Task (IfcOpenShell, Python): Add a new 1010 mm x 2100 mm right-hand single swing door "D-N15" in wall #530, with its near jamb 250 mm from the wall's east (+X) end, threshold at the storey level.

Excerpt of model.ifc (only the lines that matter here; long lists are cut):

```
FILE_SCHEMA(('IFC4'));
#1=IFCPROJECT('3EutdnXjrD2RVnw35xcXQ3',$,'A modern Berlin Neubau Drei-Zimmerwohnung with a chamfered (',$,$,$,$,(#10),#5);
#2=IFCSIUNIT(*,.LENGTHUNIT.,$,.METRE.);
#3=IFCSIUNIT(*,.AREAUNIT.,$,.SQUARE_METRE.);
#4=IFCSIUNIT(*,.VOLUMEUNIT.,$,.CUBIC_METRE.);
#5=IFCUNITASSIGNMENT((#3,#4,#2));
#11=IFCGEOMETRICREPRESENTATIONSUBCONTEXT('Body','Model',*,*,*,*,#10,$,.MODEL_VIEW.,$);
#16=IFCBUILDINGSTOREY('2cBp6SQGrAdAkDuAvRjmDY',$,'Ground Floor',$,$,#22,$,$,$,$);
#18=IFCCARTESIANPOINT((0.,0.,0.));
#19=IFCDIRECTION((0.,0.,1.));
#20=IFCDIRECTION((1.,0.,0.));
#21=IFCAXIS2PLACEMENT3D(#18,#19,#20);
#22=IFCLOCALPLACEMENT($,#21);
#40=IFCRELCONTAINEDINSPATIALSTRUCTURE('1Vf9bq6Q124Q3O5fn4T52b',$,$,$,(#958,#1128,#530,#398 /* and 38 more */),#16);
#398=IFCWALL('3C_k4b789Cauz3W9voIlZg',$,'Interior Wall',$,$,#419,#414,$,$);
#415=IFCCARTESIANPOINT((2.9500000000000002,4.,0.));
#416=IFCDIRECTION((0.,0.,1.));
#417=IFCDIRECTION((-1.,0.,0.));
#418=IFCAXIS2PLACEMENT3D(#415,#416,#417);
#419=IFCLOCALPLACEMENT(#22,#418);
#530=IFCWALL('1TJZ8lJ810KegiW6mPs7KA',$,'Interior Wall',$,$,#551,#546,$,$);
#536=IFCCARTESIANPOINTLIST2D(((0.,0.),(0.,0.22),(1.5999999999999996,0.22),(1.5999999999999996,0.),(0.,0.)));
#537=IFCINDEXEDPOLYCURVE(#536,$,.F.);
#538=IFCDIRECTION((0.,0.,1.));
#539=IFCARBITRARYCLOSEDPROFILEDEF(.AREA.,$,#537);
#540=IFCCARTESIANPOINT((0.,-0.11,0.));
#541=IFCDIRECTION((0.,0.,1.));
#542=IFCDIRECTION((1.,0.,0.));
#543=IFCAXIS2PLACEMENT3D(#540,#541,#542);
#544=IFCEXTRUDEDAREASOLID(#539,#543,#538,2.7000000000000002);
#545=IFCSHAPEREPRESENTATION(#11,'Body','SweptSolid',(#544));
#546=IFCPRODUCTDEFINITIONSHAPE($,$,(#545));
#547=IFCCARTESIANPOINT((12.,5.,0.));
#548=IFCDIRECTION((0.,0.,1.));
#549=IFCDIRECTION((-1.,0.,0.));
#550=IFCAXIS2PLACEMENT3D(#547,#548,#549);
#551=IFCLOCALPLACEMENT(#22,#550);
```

```python
import numpy as np
import ifcopenshell
import ifcopenshell.api.feature
import ifcopenshell.api.geometry
import ifcopenshell.api.root
import ifcopenshell.api.spatial
import ifcopenshell.geom
import ifcopenshell.util.element
import ifcopenshell.util.placement
import ifcopenshell.util.representation
import ifcopenshell.util.shape
import ifcopenshell.util.unit

model = ifcopenshell.open("model.ifc")
unit_scale = ifcopenshell.util.unit.calculate_unit_scale(model)
settings = ifcopenshell.geom.settings()


def volume(element):
    """Net volume in cubic metres, openings subtracted."""
    shape = ifcopenshell.geom.create_shape(settings, element)
    return ifcopenshell.util.shape.get_volume(shape.geometry)


wall = model.by_id(530)
storey = ifcopenshell.util.element.get_container(wall, ifc_class="IfcBuildingStorey")
context = ifcopenshell.util.representation.get_context(model, "Model", "Body", "MODEL_VIEW")
before = volume(wall)

width, height, from_end, sill = 1.01, 2.1, 0.25, 0.0  # metres

# The wall runs along its own X axis, and the end named is its -X end.
wall_shape = ifcopenshell.geom.create_shape(settings, wall)
x, y, z = ifcopenshell.util.shape.get_vertices(wall_shape.geometry).T
start = x.min() + from_end
face, thickness = float(y.min()), float(y.max() - y.min())
wall_matrix = ifcopenshell.util.placement.get_local_placement(wall.ObjectPlacement)
level = ifcopenshell.util.placement.get_local_placement(storey.ObjectPlacement)[2, 3]


def in_wall(x, y):
    """Placement at x, y metres in the wall's axes, at sill height."""
    matrix = wall_matrix.copy()
    matrix[:, 3] = wall_matrix @ np.array([x / unit_scale, y / unit_scale, 0.0, 1.0])
    matrix[2, 3] = level + sill / unit_scale
    return matrix


# Opening: a box that overshoots both wall faces by 50 mm.
opening = ifcopenshell.api.root.create_entity(model, ifc_class="IfcOpeningElement", predefined_type="OPENING")
box = ifcopenshell.api.geometry.add_wall_representation(
    model, context=context, length=width, height=height, thickness=thickness + 0.1
)
ifcopenshell.api.geometry.assign_representation(model, product=opening, representation=box)
ifcopenshell.api.geometry.edit_object_placement(model, product=opening, matrix=in_wall(start, face - 0.05), is_si=False)
ifcopenshell.api.feature.add_feature(model, feature=opening, element=wall)

door = ifcopenshell.api.root.create_entity(model, ifc_class="IfcDoor", name="D-N15", predefined_type="DOOR")
door.OverallWidth, door.OverallHeight = width / unit_scale, height / unit_scale
door.OperationType = "SINGLE_SWING_RIGHT"
body = ifcopenshell.api.geometry.add_door_representation(
    model,
    context=context,
    overall_width=door.OverallWidth,
    overall_height=door.OverallHeight,
    operation_type="SINGLE_SWING_RIGHT",
    lining_properties={"LiningDepth": thickness / unit_scale, "ThresholdDepth": thickness / unit_scale},
)
ifcopenshell.api.geometry.assign_representation(model, product=door, representation=body)
ifcopenshell.api.spatial.assign_container(model, products=[door], relating_structure=storey)
ifcopenshell.api.feature.add_filling(model, opening=opening, element=door)

# The lining spans the wall, so the door starts at the wall face.
ifcopenshell.api.geometry.edit_object_placement(model, product=door, matrix=in_wall(start, face), is_si=False)

after = volume(wall)

print(f"wall volume {before:.3f} -> {after:.3f} m3")

model.write("model_v2.ifc")
```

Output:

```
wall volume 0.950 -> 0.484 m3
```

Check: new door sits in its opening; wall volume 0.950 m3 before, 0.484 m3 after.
